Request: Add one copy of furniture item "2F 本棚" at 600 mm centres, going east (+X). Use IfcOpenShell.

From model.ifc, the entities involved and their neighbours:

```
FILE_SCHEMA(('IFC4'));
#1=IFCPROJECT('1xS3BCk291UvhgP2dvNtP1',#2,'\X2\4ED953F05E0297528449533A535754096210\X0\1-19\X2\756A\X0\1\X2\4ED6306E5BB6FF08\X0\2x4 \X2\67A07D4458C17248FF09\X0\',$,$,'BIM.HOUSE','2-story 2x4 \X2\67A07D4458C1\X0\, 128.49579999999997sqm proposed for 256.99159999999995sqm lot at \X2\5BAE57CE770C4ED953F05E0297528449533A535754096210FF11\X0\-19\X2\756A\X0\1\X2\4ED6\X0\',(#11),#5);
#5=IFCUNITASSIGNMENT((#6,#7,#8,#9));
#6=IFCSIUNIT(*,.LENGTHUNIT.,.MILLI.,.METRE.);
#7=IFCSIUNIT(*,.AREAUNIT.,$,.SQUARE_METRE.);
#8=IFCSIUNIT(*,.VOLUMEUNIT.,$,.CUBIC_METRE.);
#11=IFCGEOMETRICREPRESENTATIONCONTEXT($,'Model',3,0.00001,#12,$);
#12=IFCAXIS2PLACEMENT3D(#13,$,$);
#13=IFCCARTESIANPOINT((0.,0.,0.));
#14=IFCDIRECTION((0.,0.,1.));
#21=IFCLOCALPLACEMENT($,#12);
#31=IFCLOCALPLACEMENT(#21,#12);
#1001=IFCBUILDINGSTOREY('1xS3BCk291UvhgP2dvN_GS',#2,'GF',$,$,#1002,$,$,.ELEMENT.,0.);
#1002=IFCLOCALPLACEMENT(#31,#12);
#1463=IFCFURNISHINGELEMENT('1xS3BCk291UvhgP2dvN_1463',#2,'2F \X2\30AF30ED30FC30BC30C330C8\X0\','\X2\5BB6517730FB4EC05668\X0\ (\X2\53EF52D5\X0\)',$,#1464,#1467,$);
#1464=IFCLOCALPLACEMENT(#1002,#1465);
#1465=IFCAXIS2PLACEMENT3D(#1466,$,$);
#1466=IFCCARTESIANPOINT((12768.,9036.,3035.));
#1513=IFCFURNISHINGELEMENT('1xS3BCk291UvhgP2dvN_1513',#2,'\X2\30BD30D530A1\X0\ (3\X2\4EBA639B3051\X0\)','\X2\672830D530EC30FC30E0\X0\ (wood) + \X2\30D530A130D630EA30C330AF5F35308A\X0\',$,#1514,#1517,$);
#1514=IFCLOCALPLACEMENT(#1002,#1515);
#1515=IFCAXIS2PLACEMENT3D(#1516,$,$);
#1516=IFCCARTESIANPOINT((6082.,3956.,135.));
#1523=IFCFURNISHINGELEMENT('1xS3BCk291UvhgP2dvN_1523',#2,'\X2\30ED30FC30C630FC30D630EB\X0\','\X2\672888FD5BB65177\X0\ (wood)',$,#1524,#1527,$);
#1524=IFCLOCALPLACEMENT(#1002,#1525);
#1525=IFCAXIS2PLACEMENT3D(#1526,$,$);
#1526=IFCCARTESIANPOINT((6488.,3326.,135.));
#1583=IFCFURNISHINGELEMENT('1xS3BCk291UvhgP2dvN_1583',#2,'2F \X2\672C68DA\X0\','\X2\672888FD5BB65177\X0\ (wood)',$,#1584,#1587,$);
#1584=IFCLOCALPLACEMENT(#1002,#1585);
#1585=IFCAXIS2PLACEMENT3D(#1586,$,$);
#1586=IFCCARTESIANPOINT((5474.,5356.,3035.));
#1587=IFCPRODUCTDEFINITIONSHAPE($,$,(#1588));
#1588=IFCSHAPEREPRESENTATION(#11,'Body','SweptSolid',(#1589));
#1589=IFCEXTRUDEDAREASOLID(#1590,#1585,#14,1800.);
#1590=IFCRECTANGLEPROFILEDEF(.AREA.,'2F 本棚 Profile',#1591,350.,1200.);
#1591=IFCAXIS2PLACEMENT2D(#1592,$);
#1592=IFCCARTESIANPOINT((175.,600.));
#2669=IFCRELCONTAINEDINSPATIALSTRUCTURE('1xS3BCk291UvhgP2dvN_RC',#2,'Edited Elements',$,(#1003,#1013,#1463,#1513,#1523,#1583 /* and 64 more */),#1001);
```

```python
import numpy as np
import ifcopenshell
import ifcopenshell.api.geometry
import ifcopenshell.api.root
import ifcopenshell.util.element
import ifcopenshell.util.placement
import ifcopenshell.util.unit

model = ifcopenshell.open("model.ifc")
unit_scale = ifcopenshell.util.unit.calculate_unit_scale(model)


def reuse_history(source, copy):
    """copy_class also copies each property set's owner history, people and application; keep the originals."""
    for rel in copy.IsDefinedBy:
        if rel.is_a("IfcRelDefinesByProperties") and (history := rel.RelatingPropertyDefinition.OwnerHistory):
            rel.RelatingPropertyDefinition.OwnerHistory = source.OwnerHistory
            ifcopenshell.util.element.remove_deep2(model, history)


source = model.by_guid("1xS3BCk291UvhgP2dvN_1583")
base = ifcopenshell.util.placement.get_local_placement(source.ObjectPlacement)
step = np.array([1.0, 0.0, 0.0]) * 0.6 / unit_scale

for i in range(1, 2):
    copy = ifcopenshell.api.root.copy_class(model, product=source)
    copy.Representation = ifcopenshell.util.element.copy_deep(
        model, source.Representation, exclude=["IfcGeometricRepresentationContext", "IfcRepresentationMap"]
    )
    reuse_history(source, copy)
    matrix = base.copy()
    matrix[:3, 3] += i * step
    print("added at", matrix[:3, 3].round(3) + 0.0)
    ifcopenshell.api.geometry.edit_object_placement(model, product=copy, matrix=matrix, is_si=False)

model.write("model_updated.ifc")
```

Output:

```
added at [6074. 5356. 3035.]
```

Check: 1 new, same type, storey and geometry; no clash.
